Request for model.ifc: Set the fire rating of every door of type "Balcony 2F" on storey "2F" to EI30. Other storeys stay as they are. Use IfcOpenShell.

First a look at what the model holds.

```python
import ifcopenshell
import ifcopenshell.util.element

model = ifcopenshell.open("model.ifc")
print(model.schema)
storey = next(s for s in model.by_type("IfcBuildingStorey") if s.Name == "2F")
doors = [e for e in ifcopenshell.util.element.get_decomposition(storey) if e.is_a("IfcDoor")]
seen = {}
for e in doors:
    element_type = ifcopenshell.util.element.get_type(e)
    key = (element_type.Name if element_type != e and element_type else None, ifcopenshell.util.element.get_pset(e, "Pset_DoorCommon", "FireRating"))
    seen[key] = seen.get(key, 0) + 1
for (name, value), count in sorted(seen.items(), key=str):
    print(count, "x", name, "|", value)
```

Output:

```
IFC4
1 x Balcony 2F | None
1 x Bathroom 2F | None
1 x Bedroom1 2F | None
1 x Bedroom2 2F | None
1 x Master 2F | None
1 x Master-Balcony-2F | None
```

```python
import ifcopenshell
import ifcopenshell.api.pset
import ifcopenshell.util.element

model = ifcopenshell.open("model.ifc")

storey = next(s for s in model.by_type("IfcBuildingStorey") if s.Name == "2F")
doors = [e for e in ifcopenshell.util.element.get_decomposition(storey) if e.is_a("IfcDoor")]

count = 0
for e in doors:
    element_type = ifcopenshell.util.element.get_type(e)
    if element_type in (None, e) or element_type.Name != "Balcony 2F":
        continue
    # add_pset returns the element's existing set when there is one.
    pset = ifcopenshell.api.pset.add_pset(model, product=e, name="Pset_DoorCommon")
    ifcopenshell.api.pset.edit_pset(model, pset=pset, properties={"FireRating": "EI30"})
    count += 1

print(count, "doors updated")

model.write("model_updated.ifc")
```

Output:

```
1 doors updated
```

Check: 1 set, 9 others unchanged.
